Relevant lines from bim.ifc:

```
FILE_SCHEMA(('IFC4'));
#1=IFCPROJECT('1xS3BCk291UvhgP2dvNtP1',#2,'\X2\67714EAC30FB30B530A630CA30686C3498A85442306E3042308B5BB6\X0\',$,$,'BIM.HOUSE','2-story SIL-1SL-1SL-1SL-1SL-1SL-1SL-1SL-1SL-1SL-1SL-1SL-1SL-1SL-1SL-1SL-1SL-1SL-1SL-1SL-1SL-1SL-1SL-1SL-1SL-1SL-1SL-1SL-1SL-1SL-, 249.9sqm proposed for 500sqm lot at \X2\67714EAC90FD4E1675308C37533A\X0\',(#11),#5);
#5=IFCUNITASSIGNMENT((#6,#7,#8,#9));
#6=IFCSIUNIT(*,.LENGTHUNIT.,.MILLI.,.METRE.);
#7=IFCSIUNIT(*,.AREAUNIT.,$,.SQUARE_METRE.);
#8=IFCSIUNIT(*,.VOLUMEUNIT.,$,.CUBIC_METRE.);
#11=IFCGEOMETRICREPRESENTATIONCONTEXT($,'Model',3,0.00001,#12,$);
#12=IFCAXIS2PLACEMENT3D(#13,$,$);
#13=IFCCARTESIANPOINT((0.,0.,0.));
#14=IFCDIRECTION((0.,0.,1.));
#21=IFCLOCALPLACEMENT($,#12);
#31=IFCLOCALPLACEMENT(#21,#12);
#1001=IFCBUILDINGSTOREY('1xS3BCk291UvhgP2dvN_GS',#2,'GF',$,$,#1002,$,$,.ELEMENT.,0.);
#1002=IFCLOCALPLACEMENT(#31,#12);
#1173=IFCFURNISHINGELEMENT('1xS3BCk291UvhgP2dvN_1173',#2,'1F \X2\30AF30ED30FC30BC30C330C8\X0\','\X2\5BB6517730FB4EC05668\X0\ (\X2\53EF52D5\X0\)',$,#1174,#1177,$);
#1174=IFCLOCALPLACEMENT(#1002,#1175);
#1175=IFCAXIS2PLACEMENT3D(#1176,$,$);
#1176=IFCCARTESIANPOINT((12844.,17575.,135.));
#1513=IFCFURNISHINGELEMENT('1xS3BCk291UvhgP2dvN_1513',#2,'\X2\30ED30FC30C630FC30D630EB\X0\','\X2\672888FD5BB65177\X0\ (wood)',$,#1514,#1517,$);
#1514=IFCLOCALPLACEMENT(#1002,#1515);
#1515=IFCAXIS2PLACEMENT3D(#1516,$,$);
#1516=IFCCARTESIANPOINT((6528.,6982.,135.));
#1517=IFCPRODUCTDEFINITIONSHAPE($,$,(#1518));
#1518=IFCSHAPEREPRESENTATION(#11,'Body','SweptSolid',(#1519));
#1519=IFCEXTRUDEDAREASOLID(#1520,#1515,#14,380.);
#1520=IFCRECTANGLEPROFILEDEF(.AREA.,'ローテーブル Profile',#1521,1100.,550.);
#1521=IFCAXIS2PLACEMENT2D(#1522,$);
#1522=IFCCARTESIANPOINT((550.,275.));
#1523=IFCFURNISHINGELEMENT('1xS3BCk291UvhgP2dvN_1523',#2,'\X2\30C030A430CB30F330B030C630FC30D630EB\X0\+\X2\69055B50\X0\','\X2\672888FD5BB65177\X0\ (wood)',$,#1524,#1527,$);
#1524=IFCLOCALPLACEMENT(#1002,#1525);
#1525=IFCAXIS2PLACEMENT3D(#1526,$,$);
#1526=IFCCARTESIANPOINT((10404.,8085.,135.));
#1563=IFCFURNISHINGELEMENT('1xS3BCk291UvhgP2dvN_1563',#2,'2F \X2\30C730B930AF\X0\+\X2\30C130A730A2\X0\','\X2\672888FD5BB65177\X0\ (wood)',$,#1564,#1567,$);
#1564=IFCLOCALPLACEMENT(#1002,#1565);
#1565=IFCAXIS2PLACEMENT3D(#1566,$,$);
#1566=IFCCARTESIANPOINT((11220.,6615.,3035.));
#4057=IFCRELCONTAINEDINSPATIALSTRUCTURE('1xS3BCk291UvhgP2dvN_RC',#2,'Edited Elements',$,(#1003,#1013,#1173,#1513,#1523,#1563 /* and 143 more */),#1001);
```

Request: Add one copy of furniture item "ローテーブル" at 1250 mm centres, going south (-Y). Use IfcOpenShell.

```python
import numpy as np
import ifcopenshell
import ifcopenshell.api.geometry
import ifcopenshell.api.root
import ifcopenshell.util.element
import ifcopenshell.util.placement

model = ifcopenshell.open("bim.ifc")


def reuse_history(source, copy):
    """copy_class also copies each property set's owner history, people and application; keep the originals."""
    for rel in copy.IsDefinedBy:
        if rel.is_a("IfcRelDefinesByProperties") and (history := rel.RelatingPropertyDefinition.OwnerHistory):
            rel.RelatingPropertyDefinition.OwnerHistory = source.OwnerHistory
            ifcopenshell.util.element.remove_deep2(model, history)


source = model.by_guid("1xS3BCk291UvhgP2dvN_1513")
base = ifcopenshell.util.placement.get_local_placement(source.ObjectPlacement)
step = np.array([0.0, -1.0, 0.0]) * 1250.0

for i in range(1, 2):
    copy = ifcopenshell.api.root.copy_class(model, product=source)
    copy.Representation = ifcopenshell.util.element.copy_deep(
        model, source.Representation, exclude=["IfcGeometricRepresentationContext", "IfcRepresentationMap"]
    )
    reuse_history(source, copy)
    matrix = base.copy()
    matrix[:3, 3] += i * step
    print("added at", matrix[:3, 3].round(3) + 0.0)
    ifcopenshell.api.geometry.edit_object_placement(model, product=copy, matrix=matrix, is_si=False)

model.write("bim_v2.ifc")
```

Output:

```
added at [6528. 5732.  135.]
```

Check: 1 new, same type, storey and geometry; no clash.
